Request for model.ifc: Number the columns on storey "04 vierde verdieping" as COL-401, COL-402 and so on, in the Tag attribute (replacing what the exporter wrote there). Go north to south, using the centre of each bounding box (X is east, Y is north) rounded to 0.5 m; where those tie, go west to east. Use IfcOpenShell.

First a look at what the model holds.

```python
import ifcopenshell
import ifcopenshell.util.element
import ifcopenshell.util.placement

model = ifcopenshell.open("model.ifc")
print(model.schema)
storey = next(s for s in model.by_type("IfcBuildingStorey") if s.Name == "04 vierde verdieping")
columns = [e for e in ifcopenshell.util.element.get_decomposition(storey) if e.is_a("IfcColumn")]
for e in sorted(columns, key=lambda e: e.id()):
    origin = ifcopenshell.util.placement.get_local_placement(e.ObjectPlacement)[:3, 3]
    print(e.id(), e.Tag, e.Name, origin.round(2) + 0.0, sep=" | ")
```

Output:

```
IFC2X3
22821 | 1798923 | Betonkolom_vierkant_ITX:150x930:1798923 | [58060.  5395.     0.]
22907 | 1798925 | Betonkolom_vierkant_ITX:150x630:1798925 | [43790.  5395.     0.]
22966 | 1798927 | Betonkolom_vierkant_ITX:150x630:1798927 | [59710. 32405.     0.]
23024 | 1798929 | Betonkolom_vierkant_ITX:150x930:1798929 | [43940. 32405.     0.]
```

```python
import ifcopenshell
import ifcopenshell.geom
import ifcopenshell.util.element
import ifcopenshell.util.shape

model = ifcopenshell.open("model.ifc")
settings = ifcopenshell.geom.settings()
settings.set("use-world-coords", True)


def centre(element):
    shape = ifcopenshell.geom.create_shape(settings, element)
    return ifcopenshell.util.shape.get_bbox_centroid(shape.geometry)


storey = next(s for s in model.by_type("IfcBuildingStorey") if s.Name == "04 vierde verdieping")
columns = [e for e in ifcopenshell.util.element.get_decomposition(storey) if e.is_a("IfcColumn")]

# Insertion points can sit at a corner or the storey origin, so sort by the geometry (in metres).
centres = {e: centre(e) for e in columns}
columns.sort(key=lambda e: (-round(centres[e][1] / 0.5), centres[e][0]))

for i, e in enumerate(columns, start=1):
    number = f"COL-4{i:02d}"
    e.Tag = number
    print(e.id(), number)

model.write("model_rev.ifc")
```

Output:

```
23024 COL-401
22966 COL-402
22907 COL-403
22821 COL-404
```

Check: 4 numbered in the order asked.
